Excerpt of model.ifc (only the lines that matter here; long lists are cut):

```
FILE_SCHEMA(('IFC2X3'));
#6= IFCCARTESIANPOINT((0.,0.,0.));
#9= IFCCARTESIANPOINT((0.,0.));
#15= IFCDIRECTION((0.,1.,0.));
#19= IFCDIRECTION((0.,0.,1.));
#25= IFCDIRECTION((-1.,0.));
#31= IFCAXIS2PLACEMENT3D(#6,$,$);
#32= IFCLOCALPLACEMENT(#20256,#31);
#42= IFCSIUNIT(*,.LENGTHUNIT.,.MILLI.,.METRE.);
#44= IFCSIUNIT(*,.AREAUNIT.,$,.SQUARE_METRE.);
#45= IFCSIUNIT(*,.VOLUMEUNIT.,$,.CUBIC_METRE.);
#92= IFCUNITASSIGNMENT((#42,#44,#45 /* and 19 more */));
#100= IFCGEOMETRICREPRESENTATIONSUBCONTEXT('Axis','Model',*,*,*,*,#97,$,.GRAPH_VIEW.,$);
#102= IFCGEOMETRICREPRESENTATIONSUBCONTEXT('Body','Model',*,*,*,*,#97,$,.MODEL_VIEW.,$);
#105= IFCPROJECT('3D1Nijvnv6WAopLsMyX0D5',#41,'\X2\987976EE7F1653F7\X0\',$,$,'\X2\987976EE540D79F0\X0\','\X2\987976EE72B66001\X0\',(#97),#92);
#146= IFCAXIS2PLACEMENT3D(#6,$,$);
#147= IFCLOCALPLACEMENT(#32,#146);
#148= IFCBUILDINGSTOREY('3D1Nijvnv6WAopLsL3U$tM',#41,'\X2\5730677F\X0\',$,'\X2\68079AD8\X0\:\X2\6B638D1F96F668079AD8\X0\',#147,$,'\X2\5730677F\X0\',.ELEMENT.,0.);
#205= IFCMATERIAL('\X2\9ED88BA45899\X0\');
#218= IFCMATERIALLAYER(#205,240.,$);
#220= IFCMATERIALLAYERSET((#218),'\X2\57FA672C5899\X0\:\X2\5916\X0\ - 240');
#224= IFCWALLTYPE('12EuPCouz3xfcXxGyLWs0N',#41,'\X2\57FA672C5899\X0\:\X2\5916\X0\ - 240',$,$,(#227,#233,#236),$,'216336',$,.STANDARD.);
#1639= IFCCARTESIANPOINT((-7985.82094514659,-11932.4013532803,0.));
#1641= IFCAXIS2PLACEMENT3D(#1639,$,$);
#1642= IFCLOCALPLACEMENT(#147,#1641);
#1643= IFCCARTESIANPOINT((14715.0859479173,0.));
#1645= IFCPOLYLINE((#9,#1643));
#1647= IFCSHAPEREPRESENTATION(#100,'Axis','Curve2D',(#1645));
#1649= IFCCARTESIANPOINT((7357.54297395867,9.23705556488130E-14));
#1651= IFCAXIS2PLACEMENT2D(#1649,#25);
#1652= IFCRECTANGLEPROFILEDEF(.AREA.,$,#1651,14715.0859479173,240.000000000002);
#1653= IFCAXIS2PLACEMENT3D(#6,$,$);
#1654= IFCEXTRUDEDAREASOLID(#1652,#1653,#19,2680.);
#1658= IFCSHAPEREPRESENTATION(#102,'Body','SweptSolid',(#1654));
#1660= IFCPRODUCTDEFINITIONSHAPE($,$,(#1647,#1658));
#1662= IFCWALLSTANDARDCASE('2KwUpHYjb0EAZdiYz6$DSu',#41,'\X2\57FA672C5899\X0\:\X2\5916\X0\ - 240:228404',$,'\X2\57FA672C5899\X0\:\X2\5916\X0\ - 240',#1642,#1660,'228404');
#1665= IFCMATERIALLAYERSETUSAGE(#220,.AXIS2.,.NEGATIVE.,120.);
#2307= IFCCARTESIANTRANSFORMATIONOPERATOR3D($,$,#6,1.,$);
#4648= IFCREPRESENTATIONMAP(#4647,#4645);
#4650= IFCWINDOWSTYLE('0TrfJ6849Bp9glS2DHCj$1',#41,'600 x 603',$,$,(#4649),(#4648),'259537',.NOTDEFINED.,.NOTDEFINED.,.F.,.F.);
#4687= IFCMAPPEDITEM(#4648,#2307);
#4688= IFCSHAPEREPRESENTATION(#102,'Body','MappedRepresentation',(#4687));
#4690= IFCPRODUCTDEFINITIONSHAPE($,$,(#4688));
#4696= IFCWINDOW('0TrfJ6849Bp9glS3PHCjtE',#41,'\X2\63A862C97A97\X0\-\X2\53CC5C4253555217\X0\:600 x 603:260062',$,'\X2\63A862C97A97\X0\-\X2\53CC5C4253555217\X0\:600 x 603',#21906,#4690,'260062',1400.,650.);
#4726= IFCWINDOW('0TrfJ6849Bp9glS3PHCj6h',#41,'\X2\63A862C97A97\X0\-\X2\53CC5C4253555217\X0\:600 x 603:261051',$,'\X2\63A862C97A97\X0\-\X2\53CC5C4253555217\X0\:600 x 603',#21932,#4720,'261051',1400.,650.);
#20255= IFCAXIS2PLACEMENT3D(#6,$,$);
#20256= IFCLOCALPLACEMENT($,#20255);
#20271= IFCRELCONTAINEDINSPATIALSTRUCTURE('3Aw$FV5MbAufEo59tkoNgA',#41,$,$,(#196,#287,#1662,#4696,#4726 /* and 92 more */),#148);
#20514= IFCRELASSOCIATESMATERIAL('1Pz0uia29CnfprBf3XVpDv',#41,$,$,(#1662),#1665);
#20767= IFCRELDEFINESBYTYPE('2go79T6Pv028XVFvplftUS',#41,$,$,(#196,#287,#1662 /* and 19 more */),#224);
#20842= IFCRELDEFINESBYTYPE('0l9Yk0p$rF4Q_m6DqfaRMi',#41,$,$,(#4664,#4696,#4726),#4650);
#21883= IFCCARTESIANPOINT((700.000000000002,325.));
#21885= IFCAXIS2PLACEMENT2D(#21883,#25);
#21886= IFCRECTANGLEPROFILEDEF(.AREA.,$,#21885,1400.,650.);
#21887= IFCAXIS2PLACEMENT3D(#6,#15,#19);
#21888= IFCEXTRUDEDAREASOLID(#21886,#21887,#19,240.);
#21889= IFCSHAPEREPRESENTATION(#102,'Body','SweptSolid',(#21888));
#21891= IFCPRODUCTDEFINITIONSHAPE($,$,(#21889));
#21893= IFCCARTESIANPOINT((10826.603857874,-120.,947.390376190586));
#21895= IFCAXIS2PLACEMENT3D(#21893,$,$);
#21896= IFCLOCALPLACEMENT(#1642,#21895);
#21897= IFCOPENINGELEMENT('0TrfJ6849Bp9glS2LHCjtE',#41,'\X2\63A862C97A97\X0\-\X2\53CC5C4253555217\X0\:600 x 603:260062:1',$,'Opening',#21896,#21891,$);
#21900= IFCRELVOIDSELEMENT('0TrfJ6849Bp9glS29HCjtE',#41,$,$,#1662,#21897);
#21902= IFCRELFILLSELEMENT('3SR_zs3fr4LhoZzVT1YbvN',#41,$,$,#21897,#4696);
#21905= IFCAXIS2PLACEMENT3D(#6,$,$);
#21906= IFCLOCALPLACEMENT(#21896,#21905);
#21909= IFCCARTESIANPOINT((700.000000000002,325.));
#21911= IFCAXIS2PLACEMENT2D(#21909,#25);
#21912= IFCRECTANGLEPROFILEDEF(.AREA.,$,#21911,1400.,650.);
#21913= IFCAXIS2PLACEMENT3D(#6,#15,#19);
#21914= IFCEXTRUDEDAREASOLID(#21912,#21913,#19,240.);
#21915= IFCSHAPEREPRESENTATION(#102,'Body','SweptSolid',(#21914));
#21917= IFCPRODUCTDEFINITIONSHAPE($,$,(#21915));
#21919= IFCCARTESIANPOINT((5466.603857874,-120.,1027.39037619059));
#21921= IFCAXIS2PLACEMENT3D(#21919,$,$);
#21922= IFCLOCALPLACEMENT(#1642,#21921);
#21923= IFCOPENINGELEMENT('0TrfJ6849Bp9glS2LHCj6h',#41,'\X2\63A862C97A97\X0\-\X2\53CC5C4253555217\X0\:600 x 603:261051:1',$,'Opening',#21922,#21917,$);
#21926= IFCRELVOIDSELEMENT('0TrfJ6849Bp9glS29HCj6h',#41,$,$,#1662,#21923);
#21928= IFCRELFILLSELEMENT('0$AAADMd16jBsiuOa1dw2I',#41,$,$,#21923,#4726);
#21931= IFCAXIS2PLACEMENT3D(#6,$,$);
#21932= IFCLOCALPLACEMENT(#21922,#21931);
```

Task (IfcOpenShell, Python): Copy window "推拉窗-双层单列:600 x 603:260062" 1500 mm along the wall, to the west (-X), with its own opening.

```python
import ifcopenshell
import ifcopenshell.api.feature
import ifcopenshell.api.geometry
import ifcopenshell.api.root
import ifcopenshell.geom
import ifcopenshell.util.element
import ifcopenshell.util.placement
import ifcopenshell.util.shape
import ifcopenshell.util.unit

model = ifcopenshell.open("model.ifc")
unit_scale = ifcopenshell.util.unit.calculate_unit_scale(model)
settings = ifcopenshell.geom.settings()


def volume(element):
    """Net volume in cubic metres, openings subtracted."""
    shape = ifcopenshell.geom.create_shape(settings, element)
    return ifcopenshell.util.shape.get_volume(shape.geometry)


def reuse_history(source, copy):
    """copy_class also copies each property set's owner history, people and application; keep the originals."""
    for rel in copy.IsDefinedBy:
        if rel.is_a("IfcRelDefinesByProperties") and (history := rel.RelatingPropertyDefinition.OwnerHistory):
            rel.RelatingPropertyDefinition.OwnerHistory = source.OwnerHistory
            ifcopenshell.util.element.remove_deep2(model, history)


window = model.by_guid("0TrfJ6849Bp9glS3PHCjtE")
opening = window.FillsVoids[0].RelatingOpeningElement
wall = opening.VoidsElements[0].RelatingBuildingElement
before = volume(wall)
shift = ifcopenshell.util.placement.get_local_placement(wall.ObjectPlacement)[:3, 0] * -1.5 / unit_scale

# copy_class copies the void relationship, type, container and properties, but no geometry.
new_opening = ifcopenshell.api.root.copy_class(model, product=opening)
new_opening.Representation = ifcopenshell.util.element.copy_deep(
    model, opening.Representation, exclude=["IfcGeometricRepresentationContext", "IfcRepresentationMap"]
)
new_opening.Name = "推拉窗-双层单列:600 x 603"
new_window = ifcopenshell.api.root.copy_class(model, product=window)
new_window.Representation = ifcopenshell.util.element.copy_deep(
    model, window.Representation, exclude=["IfcGeometricRepresentationContext", "IfcRepresentationMap"]
)
new_window.Name = "推拉窗-双层单列:600 x 603"
new_window.Tag = None
reuse_history(window, new_window)
fills = ifcopenshell.api.feature.add_filling(model, opening=new_opening, element=new_window)
fills.OwnerHistory = new_window.OwnerHistory  # required in IFC2X3

for old, new in ((opening, new_opening), (window, new_window)):
    matrix = ifcopenshell.util.placement.get_local_placement(old.ObjectPlacement)
    matrix[:3, 3] += shift
    ifcopenshell.api.geometry.edit_object_placement(model, product=new, matrix=matrix, is_si=False)

after = volume(wall)

print(f"wall volume {before:.3f} -> {after:.3f} m3")

model.write("model-out.ifc")
```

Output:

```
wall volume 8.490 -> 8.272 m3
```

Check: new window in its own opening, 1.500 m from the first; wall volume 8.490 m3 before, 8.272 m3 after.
